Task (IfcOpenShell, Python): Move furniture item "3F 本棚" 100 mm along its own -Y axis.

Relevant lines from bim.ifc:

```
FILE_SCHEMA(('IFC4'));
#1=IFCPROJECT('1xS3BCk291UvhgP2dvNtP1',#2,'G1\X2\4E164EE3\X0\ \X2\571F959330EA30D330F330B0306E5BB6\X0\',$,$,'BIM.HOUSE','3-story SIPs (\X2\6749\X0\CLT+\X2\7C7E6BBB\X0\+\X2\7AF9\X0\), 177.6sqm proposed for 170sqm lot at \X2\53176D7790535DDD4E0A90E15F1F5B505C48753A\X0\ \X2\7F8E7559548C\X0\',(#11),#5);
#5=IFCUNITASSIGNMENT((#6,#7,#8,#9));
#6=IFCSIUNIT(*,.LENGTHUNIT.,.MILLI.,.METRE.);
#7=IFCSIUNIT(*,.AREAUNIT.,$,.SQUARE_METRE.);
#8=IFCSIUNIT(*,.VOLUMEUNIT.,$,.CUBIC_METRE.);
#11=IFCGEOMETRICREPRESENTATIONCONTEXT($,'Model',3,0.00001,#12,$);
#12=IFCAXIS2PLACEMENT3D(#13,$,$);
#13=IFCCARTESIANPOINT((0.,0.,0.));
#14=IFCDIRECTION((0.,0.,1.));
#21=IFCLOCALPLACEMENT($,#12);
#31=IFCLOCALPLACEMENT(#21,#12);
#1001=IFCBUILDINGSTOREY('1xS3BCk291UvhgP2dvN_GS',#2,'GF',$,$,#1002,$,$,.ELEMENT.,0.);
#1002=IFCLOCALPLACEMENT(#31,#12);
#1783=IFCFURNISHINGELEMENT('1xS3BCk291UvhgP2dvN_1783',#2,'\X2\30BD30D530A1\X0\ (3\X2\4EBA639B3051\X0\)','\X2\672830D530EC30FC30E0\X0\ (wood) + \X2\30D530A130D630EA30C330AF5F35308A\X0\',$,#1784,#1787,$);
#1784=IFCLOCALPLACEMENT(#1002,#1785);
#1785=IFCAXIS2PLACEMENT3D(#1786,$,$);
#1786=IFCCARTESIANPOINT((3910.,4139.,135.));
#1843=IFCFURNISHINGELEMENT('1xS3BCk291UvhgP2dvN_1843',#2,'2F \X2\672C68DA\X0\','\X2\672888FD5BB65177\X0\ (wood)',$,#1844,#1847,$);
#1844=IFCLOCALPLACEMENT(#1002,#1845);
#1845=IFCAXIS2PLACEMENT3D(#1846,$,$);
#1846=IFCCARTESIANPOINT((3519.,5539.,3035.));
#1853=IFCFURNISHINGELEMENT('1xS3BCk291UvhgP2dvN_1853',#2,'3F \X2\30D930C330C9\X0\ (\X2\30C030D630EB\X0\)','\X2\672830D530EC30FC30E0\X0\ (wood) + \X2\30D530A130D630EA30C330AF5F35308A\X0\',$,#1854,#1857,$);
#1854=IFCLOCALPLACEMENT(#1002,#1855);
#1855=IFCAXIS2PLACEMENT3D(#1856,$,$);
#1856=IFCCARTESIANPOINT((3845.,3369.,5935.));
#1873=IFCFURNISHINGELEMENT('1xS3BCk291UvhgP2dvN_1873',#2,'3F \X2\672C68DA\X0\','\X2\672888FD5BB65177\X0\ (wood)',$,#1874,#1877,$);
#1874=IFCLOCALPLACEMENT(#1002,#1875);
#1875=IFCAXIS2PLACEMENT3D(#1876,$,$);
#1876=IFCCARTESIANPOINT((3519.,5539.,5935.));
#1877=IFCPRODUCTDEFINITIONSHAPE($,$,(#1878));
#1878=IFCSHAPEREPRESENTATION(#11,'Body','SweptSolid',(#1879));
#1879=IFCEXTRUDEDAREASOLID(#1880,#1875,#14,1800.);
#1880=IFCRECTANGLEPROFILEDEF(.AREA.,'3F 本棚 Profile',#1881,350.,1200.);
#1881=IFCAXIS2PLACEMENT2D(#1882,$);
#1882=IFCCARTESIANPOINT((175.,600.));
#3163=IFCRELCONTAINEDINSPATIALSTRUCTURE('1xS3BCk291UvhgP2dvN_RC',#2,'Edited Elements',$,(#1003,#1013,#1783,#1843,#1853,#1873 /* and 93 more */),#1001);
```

```python
import ifcopenshell
import ifcopenshell.api.geometry
import ifcopenshell.util.placement

model = ifcopenshell.open("bim.ifc")

item = model.by_guid("1xS3BCk291UvhgP2dvN_1873")
matrix = ifcopenshell.util.placement.get_local_placement(item.ObjectPlacement)
matrix[:3, 3] -= matrix[:3, 1] * 100.0
ifcopenshell.api.geometry.edit_object_placement(model, product=item, matrix=matrix, is_si=False)

print(ifcopenshell.util.placement.get_local_placement(item.ObjectPlacement).round(3) + 0.0)

model.write("bim_v2.ifc")
```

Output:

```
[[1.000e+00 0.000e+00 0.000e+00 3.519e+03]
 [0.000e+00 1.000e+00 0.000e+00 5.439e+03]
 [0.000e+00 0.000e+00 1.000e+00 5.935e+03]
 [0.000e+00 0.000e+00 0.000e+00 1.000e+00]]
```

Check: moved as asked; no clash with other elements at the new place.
